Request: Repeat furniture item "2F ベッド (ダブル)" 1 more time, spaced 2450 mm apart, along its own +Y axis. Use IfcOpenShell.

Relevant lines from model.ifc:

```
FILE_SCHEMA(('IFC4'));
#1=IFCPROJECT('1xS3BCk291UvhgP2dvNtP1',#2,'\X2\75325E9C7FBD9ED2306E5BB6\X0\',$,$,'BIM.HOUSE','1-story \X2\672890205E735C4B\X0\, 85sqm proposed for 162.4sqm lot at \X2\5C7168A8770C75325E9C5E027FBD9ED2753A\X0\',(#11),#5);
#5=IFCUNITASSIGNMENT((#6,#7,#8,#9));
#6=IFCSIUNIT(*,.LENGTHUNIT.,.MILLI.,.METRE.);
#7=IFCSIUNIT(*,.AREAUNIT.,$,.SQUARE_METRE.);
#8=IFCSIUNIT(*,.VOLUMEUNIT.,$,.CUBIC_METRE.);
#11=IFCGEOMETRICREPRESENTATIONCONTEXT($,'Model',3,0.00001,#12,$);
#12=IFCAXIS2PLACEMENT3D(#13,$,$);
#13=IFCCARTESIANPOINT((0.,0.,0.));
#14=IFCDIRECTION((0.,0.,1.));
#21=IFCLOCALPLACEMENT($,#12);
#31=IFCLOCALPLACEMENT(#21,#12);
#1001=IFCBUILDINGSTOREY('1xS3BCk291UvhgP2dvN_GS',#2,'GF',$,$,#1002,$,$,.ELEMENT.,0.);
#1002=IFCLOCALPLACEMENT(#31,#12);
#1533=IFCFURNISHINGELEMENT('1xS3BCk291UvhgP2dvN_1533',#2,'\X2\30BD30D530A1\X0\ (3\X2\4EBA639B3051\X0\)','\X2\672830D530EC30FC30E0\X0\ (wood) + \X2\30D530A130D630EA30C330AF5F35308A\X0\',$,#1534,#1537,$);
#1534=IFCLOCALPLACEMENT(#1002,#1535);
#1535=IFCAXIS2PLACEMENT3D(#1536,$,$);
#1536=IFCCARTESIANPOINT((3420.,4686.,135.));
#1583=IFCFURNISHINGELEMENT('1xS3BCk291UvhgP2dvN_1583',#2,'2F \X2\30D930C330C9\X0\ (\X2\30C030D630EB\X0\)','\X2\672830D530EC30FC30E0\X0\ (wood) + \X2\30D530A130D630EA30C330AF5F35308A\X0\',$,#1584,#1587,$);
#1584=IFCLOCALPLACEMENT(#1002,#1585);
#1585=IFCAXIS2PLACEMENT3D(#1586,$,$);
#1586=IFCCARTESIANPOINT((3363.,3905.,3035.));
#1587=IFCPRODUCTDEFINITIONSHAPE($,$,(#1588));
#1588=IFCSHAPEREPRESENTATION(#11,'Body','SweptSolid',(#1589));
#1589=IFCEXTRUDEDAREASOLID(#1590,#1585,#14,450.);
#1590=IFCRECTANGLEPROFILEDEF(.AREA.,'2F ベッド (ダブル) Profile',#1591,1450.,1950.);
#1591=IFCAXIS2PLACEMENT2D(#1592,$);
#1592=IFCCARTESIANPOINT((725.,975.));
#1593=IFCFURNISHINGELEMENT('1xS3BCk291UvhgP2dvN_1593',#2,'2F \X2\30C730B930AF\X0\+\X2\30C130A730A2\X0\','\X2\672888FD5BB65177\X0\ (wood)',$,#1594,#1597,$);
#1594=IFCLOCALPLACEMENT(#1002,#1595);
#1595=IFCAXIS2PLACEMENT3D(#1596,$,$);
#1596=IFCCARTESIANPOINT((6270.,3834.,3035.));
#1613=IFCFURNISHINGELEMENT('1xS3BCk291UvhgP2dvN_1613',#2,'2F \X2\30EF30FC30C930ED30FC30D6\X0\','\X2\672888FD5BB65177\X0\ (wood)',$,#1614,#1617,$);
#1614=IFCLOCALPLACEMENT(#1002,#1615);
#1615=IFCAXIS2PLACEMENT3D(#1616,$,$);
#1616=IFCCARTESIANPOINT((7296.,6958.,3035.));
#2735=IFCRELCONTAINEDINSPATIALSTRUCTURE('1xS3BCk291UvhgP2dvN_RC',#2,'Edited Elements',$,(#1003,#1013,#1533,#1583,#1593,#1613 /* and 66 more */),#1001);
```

```python
import ifcopenshell
import ifcopenshell.api.geometry
import ifcopenshell.api.root
import ifcopenshell.util.element
import ifcopenshell.util.placement
import ifcopenshell.util.unit

model = ifcopenshell.open("model.ifc")
unit_scale = ifcopenshell.util.unit.calculate_unit_scale(model)


def reuse_history(source, copy):
    """copy_class also copies each property set's owner history, people and application; keep the originals."""
    for rel in copy.IsDefinedBy:
        if rel.is_a("IfcRelDefinesByProperties") and (history := rel.RelatingPropertyDefinition.OwnerHistory):
            rel.RelatingPropertyDefinition.OwnerHistory = source.OwnerHistory
            ifcopenshell.util.element.remove_deep2(model, history)


source = model.by_id(1583)
base = ifcopenshell.util.placement.get_local_placement(source.ObjectPlacement)
step = base[:3, 1] * 2.45 / unit_scale

for i in range(1, 2):
    copy = ifcopenshell.api.root.copy_class(model, product=source)
    copy.Representation = ifcopenshell.util.element.copy_deep(
        model, source.Representation, exclude=["IfcGeometricRepresentationContext", "IfcRepresentationMap"]
    )
    reuse_history(source, copy)
    matrix = base.copy()
    matrix[:3, 3] += i * step
    print("added at", matrix[:3, 3].round(3) + 0.0)
    ifcopenshell.api.geometry.edit_object_placement(model, product=copy, matrix=matrix, is_si=False)

model.write("model-out.ifc")
```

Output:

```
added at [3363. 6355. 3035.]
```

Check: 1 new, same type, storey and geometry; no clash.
